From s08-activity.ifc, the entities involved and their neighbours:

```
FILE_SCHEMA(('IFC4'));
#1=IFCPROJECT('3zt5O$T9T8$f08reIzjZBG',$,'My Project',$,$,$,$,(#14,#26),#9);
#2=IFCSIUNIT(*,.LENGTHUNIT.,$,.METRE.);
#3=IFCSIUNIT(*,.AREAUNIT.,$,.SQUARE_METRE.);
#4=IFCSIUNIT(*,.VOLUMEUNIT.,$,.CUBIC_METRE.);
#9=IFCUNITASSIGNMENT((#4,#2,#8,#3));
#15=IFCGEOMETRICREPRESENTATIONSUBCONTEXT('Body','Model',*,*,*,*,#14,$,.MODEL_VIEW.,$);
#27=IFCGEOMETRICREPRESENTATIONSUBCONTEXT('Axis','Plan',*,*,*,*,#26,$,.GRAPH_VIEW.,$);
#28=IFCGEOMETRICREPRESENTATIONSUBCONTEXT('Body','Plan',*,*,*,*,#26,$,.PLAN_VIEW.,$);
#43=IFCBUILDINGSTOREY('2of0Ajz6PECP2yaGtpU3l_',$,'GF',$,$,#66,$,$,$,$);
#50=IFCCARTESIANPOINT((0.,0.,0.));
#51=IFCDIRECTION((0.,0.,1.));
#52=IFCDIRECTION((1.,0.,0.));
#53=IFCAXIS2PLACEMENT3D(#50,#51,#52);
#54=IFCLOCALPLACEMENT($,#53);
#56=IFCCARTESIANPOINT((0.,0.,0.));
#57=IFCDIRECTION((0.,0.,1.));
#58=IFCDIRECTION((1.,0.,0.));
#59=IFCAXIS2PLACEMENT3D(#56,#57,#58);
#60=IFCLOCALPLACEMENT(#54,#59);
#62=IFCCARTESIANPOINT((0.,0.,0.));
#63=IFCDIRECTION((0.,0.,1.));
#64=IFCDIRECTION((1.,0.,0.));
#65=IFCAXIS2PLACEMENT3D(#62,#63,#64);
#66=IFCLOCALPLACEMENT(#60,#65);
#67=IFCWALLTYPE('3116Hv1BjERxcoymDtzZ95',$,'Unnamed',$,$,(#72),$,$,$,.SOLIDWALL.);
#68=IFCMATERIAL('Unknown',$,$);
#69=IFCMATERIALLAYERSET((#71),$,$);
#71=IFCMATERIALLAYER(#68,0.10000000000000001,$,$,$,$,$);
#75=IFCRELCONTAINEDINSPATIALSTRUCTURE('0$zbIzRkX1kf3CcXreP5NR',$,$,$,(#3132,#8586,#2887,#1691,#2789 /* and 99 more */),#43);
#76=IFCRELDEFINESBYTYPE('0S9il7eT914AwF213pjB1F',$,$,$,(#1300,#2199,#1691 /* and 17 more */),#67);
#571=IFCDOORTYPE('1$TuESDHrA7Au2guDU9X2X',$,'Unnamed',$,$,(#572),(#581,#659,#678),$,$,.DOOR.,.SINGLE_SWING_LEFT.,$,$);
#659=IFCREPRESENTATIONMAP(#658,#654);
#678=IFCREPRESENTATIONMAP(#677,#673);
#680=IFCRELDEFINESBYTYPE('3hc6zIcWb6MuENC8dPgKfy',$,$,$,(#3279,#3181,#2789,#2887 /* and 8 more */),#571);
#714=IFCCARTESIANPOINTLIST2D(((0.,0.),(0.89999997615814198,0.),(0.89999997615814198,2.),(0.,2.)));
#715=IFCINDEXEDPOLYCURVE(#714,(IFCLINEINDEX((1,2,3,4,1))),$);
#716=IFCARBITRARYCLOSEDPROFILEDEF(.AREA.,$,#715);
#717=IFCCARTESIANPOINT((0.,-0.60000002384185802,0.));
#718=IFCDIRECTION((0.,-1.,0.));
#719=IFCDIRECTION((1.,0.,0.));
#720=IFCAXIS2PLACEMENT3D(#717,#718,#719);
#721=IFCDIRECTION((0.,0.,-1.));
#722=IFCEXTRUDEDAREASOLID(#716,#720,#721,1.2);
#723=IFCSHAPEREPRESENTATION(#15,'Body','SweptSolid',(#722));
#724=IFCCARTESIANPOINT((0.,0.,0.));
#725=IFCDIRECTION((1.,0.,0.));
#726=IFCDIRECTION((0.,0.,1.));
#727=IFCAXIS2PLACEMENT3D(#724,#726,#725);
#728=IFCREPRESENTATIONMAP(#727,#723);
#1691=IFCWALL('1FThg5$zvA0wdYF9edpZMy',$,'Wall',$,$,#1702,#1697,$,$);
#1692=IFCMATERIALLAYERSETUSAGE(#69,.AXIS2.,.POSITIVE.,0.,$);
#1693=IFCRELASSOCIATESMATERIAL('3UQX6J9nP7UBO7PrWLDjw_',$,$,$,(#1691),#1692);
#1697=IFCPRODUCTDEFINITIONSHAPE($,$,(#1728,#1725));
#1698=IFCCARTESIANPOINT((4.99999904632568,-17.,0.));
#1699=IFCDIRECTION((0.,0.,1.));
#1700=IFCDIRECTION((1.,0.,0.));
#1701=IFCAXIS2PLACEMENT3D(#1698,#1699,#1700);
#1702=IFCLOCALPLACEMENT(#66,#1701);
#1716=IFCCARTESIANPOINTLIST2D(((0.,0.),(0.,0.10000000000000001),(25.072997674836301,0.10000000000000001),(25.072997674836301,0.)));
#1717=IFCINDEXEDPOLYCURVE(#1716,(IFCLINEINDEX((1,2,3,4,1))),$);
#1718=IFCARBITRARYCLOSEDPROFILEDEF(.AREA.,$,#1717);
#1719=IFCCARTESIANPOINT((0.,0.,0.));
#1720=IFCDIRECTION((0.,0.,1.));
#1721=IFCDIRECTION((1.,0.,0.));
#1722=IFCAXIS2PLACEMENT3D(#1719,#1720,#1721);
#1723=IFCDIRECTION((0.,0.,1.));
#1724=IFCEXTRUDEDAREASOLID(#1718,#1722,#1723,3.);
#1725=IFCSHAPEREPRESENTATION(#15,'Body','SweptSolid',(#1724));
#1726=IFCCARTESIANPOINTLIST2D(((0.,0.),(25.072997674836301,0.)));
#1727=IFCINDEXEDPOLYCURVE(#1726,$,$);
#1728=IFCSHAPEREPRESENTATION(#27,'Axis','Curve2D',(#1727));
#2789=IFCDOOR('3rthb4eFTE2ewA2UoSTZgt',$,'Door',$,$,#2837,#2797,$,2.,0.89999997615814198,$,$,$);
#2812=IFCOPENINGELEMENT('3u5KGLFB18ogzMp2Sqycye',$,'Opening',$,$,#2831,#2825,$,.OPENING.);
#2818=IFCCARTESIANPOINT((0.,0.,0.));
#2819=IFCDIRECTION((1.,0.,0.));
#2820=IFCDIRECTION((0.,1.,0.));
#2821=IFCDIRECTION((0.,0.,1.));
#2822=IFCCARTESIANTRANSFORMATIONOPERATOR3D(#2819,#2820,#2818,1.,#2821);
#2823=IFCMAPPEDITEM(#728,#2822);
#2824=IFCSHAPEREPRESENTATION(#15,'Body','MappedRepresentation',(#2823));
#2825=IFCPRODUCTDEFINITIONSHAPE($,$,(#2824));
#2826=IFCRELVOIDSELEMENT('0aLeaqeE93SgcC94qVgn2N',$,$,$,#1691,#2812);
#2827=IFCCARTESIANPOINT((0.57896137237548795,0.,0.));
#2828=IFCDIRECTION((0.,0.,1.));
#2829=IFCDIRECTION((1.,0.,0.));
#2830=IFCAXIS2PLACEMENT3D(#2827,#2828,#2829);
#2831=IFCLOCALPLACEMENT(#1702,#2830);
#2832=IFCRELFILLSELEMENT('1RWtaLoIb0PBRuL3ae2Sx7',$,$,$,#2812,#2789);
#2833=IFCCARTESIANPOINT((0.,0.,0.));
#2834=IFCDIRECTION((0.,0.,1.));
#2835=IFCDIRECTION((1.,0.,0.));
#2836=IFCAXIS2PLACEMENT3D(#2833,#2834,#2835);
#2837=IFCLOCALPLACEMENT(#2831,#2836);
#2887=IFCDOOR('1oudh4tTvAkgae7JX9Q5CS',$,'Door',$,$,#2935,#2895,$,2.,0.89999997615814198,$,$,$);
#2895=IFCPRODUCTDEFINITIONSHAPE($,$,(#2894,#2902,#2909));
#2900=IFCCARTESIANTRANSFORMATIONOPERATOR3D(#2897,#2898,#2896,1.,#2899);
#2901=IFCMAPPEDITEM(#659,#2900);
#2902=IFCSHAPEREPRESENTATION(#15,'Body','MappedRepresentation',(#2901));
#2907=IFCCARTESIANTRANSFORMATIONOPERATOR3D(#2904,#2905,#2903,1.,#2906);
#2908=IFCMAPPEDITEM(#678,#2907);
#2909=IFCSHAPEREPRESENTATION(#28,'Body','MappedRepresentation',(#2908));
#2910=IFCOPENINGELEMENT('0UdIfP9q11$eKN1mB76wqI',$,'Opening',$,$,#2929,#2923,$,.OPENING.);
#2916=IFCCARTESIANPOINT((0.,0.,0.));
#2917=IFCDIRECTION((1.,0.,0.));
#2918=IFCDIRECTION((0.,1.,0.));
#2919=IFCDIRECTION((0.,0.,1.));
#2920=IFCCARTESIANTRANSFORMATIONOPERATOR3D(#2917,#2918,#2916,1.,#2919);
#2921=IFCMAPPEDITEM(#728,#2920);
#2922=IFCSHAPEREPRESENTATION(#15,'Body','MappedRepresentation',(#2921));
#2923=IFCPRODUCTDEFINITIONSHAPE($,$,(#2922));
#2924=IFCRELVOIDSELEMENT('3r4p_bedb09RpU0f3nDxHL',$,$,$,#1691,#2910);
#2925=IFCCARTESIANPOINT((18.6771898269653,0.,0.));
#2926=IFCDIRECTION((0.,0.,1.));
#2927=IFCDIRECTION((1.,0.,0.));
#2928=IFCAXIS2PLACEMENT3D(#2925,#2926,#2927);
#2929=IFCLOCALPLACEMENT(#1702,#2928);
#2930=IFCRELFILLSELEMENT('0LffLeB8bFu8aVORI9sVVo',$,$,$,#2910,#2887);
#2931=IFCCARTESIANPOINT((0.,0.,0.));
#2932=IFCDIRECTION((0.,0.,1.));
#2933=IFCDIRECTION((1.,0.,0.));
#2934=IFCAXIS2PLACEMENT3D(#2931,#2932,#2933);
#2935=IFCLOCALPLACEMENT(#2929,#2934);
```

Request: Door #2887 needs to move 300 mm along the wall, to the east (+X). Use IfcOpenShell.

```python
import ifcopenshell
import ifcopenshell.api.geometry
import ifcopenshell.util.placement
import ifcopenshell.util.unit

model = ifcopenshell.open("s08-activity.ifc")
unit_scale = ifcopenshell.util.unit.calculate_unit_scale(model)

door = model.by_guid("1oudh4tTvAkgae7JX9Q5CS")
opening = door.FillsVoids[0].RelatingOpeningElement
wall = opening.VoidsElements[0].RelatingBuildingElement

wall_matrix = ifcopenshell.util.placement.get_local_placement(wall.ObjectPlacement)
shift = wall_matrix[:3, 0] * 0.3 / unit_scale
before = ifcopenshell.util.placement.get_local_placement(door.ObjectPlacement)[:3, 3].copy()

# The door is placed relative to its opening, so it follows when the opening moves.
matrix = ifcopenshell.util.placement.get_local_placement(opening.ObjectPlacement)
matrix[:3, 3] += shift
ifcopenshell.api.geometry.edit_object_placement(
    model, product=opening, matrix=matrix, is_si=False, should_transform_children=True
)

after = ifcopenshell.util.placement.get_local_placement(door.ObjectPlacement)[:3, 3]
print("door moved by", (after - before).round(3) + 0.0)

model.write("s08-activity_rev.ifc")
```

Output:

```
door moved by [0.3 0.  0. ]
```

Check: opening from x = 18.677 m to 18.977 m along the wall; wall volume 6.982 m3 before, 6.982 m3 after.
